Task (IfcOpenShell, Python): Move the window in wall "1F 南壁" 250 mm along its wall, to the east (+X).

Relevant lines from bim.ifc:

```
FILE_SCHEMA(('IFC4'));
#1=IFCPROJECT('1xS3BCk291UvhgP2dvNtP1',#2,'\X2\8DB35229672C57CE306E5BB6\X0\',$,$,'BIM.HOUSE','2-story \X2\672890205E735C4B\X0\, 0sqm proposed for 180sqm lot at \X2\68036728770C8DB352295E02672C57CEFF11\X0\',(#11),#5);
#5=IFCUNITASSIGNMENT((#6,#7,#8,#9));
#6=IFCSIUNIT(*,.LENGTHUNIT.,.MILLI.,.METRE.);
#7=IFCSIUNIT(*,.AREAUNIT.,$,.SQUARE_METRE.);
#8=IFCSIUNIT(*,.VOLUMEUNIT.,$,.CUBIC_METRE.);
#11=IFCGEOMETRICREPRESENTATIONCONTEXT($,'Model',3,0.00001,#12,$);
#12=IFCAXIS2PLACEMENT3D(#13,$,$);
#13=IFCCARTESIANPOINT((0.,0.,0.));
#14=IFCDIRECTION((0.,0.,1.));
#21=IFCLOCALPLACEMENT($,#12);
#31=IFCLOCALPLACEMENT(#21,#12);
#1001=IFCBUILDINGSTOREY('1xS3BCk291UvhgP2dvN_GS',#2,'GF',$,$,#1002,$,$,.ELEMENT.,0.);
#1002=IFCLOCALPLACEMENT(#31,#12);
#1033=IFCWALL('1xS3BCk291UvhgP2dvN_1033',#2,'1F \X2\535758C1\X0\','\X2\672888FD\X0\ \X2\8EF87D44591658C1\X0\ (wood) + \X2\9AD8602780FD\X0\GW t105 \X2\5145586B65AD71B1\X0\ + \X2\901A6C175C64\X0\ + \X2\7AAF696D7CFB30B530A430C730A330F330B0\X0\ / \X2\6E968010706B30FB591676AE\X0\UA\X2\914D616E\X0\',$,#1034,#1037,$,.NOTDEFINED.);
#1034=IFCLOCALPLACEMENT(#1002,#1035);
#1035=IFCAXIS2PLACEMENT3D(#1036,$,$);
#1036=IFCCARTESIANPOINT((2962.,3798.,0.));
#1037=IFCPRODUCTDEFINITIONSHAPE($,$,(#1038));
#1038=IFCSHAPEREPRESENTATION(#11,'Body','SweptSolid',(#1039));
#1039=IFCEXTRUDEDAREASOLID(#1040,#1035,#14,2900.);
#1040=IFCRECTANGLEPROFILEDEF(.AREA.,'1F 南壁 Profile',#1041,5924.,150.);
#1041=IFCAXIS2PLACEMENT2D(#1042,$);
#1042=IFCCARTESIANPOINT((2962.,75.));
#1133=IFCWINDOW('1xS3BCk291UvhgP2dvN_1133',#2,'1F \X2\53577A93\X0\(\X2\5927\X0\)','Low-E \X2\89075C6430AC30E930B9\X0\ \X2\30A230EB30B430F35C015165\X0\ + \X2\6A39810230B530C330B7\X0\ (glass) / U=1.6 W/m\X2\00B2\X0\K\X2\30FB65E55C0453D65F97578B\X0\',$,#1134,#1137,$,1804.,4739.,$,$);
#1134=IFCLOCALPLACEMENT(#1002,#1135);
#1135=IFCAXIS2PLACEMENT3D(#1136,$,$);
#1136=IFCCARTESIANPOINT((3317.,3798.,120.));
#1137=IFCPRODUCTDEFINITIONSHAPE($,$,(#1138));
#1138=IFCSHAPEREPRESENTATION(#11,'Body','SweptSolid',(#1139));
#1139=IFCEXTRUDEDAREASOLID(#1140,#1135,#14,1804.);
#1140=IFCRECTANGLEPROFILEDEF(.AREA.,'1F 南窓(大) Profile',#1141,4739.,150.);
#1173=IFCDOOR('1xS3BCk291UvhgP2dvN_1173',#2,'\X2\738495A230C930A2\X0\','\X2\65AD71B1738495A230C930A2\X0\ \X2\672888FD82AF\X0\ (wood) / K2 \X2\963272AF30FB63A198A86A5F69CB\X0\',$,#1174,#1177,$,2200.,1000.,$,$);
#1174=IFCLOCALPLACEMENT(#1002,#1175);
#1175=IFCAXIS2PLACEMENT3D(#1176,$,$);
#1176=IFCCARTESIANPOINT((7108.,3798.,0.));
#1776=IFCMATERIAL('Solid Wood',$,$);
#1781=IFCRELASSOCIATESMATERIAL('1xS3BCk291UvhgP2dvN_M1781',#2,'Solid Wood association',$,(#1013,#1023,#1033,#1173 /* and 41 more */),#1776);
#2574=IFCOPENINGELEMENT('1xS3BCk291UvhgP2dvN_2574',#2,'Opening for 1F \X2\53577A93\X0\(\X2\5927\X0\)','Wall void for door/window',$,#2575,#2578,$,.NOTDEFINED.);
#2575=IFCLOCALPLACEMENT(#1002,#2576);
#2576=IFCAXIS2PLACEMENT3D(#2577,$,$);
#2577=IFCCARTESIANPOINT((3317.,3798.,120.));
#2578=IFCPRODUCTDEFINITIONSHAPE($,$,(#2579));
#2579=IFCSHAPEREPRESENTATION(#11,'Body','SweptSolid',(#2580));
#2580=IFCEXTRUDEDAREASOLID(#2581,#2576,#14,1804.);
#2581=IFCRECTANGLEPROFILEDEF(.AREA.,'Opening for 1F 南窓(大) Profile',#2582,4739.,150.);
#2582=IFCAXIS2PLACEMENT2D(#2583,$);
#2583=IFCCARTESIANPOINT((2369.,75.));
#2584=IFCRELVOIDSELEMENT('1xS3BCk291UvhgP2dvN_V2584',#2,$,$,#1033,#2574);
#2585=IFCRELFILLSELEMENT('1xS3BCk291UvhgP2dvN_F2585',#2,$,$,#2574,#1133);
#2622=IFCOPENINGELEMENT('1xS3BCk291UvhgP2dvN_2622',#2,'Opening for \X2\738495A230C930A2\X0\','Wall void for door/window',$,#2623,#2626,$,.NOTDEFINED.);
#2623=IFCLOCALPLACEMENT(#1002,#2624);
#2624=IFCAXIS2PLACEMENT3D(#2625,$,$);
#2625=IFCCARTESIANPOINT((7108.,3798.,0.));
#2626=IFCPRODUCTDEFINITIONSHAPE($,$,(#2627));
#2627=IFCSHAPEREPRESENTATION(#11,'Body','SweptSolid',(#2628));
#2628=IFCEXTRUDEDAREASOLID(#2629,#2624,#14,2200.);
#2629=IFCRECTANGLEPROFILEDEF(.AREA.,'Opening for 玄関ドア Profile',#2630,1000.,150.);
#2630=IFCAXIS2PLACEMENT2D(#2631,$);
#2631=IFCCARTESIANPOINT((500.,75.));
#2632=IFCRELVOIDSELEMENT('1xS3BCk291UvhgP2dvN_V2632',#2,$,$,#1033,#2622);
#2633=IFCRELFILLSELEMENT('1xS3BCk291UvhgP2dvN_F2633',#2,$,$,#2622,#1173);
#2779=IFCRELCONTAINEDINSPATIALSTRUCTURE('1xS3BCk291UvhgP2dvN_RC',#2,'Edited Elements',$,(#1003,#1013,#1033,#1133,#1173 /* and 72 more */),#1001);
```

```python
import ifcopenshell
import ifcopenshell.api.geometry
import ifcopenshell.util.placement

model = ifcopenshell.open("bim.ifc")

window = model.by_guid("1xS3BCk291UvhgP2dvN_1133")
opening = window.FillsVoids[0].RelatingOpeningElement
wall = opening.VoidsElements[0].RelatingBuildingElement

wall_matrix = ifcopenshell.util.placement.get_local_placement(wall.ObjectPlacement)
shift = wall_matrix[:3, 0] * 250.0
before = ifcopenshell.util.placement.get_local_placement(window.ObjectPlacement)[:3, 3].copy()

# The window is not placed relative to its opening, so move both.
for product in (opening, window):
    matrix = ifcopenshell.util.placement.get_local_placement(product.ObjectPlacement)
    matrix[:3, 3] += shift
    ifcopenshell.api.geometry.edit_object_placement(model, product=product, matrix=matrix, is_si=False)

after = ifcopenshell.util.placement.get_local_placement(window.ObjectPlacement)[:3, 3]
print("window moved by", (after - before).round(3) + 0.0)

model.write("bim_v2.ifc")
```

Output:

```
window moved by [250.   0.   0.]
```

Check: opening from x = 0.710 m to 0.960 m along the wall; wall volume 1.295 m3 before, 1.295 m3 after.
